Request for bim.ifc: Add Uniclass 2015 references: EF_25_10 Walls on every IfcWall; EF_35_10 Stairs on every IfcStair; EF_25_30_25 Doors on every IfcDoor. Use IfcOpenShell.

First a look at what the model holds.

```python
import ifcopenshell

model = ifcopenshell.open("bim.ifc")
print(model.schema)
print("classifications:", [c.Name for c in model.by_type("IfcClassification")])
for ifc_class in ("IfcDoor", "IfcRoof", "IfcStair", "IfcWall", "IfcWindow"):
    print(ifc_class, len(model.by_type(ifc_class)))
```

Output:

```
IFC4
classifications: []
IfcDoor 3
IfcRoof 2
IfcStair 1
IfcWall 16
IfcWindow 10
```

```python
import ifcopenshell
import ifcopenshell.api.classification

model = ifcopenshell.open("bim.ifc")

system = ifcopenshell.api.classification.add_classification(model, classification="Uniclass 2015")

codes = {
    "IfcWall": ("EF_25_10", "Walls"),
    "IfcStair": ("EF_35_10", "Stairs"),
    "IfcDoor": ("EF_25_30_25", "Doors"),
}
for ifc_class, (code, name) in codes.items():
    products = model.by_type(ifc_class)
    ifcopenshell.api.classification.add_reference(
        model, products=products, classification=system, identification=code, name=name
    )
    print(code, len(products))

model.write("bim_updated.ifc")
```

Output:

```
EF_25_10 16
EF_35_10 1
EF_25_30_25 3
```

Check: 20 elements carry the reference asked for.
